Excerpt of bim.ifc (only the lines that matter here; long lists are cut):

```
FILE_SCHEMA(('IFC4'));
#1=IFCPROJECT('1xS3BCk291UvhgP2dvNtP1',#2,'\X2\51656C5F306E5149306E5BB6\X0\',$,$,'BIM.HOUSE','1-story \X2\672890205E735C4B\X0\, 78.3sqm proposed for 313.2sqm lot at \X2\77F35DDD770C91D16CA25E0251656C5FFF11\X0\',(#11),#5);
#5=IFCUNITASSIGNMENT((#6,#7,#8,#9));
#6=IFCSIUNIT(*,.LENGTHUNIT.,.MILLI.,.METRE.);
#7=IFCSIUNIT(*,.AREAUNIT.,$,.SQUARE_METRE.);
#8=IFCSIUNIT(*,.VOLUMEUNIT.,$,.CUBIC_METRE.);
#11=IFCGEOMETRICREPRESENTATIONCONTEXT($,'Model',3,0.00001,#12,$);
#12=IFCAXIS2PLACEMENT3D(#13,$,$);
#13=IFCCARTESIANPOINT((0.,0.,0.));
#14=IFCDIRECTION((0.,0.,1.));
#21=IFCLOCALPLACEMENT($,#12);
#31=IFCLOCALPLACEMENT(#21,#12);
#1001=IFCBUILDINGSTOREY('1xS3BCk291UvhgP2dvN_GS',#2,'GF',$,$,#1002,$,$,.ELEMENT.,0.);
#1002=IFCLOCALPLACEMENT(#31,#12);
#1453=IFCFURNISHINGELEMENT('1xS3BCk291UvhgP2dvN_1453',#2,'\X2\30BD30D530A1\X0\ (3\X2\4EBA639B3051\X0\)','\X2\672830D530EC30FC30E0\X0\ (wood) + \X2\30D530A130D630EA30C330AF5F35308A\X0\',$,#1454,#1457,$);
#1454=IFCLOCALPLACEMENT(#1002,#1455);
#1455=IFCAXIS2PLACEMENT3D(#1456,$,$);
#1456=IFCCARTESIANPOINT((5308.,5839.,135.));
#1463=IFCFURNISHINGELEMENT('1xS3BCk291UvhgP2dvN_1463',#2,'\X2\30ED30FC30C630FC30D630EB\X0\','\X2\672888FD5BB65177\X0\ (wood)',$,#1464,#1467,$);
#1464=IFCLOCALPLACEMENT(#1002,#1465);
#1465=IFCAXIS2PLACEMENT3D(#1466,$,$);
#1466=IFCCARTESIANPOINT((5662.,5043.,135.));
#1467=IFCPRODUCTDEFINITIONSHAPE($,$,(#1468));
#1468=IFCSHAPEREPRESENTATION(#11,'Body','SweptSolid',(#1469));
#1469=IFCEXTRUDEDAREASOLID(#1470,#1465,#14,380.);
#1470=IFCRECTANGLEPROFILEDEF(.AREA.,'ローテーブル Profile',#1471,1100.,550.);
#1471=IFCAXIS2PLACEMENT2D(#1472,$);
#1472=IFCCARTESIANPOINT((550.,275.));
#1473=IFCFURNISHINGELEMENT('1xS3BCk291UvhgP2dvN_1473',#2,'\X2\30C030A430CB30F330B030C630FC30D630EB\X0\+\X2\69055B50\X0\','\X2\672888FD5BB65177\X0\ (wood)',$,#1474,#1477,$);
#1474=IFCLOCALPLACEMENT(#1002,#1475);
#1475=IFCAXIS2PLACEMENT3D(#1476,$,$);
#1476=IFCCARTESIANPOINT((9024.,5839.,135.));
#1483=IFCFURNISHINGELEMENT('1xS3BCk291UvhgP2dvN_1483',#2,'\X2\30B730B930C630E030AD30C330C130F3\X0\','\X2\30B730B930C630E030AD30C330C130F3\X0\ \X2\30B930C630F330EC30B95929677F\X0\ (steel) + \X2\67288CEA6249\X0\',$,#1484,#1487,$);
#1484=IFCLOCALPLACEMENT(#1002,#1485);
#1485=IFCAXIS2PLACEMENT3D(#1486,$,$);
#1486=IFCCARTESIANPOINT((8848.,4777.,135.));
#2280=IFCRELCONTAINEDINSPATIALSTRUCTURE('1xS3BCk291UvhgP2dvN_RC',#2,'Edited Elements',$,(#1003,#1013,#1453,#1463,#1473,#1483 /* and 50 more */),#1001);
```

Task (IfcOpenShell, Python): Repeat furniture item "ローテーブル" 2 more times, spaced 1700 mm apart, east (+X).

```python
import numpy as np
import ifcopenshell
import ifcopenshell.api.geometry
import ifcopenshell.api.root
import ifcopenshell.util.element
import ifcopenshell.util.placement

model = ifcopenshell.open("bim.ifc")


def reuse_history(source, copy):
    """copy_class also copies each property set's owner history, people and application; keep the originals."""
    for rel in copy.IsDefinedBy:
        if rel.is_a("IfcRelDefinesByProperties") and (history := rel.RelatingPropertyDefinition.OwnerHistory):
            rel.RelatingPropertyDefinition.OwnerHistory = source.OwnerHistory
            ifcopenshell.util.element.remove_deep2(model, history)


source = model.by_guid("1xS3BCk291UvhgP2dvN_1463")
base = ifcopenshell.util.placement.get_local_placement(source.ObjectPlacement)
step = np.array([1.0, 0.0, 0.0]) * 1700.0

for i in range(1, 3):
    copy = ifcopenshell.api.root.copy_class(model, product=source)
    copy.Representation = ifcopenshell.util.element.copy_deep(
        model, source.Representation, exclude=["IfcGeometricRepresentationContext", "IfcRepresentationMap"]
    )
    reuse_history(source, copy)
    matrix = base.copy()
    matrix[:3, 3] += i * step
    print("added at", matrix[:3, 3].round(3) + 0.0)
    ifcopenshell.api.geometry.edit_object_placement(model, product=copy, matrix=matrix, is_si=False)

model.write("bim_updated.ifc")
```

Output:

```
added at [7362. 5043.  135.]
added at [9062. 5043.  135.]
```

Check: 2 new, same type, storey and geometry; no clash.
